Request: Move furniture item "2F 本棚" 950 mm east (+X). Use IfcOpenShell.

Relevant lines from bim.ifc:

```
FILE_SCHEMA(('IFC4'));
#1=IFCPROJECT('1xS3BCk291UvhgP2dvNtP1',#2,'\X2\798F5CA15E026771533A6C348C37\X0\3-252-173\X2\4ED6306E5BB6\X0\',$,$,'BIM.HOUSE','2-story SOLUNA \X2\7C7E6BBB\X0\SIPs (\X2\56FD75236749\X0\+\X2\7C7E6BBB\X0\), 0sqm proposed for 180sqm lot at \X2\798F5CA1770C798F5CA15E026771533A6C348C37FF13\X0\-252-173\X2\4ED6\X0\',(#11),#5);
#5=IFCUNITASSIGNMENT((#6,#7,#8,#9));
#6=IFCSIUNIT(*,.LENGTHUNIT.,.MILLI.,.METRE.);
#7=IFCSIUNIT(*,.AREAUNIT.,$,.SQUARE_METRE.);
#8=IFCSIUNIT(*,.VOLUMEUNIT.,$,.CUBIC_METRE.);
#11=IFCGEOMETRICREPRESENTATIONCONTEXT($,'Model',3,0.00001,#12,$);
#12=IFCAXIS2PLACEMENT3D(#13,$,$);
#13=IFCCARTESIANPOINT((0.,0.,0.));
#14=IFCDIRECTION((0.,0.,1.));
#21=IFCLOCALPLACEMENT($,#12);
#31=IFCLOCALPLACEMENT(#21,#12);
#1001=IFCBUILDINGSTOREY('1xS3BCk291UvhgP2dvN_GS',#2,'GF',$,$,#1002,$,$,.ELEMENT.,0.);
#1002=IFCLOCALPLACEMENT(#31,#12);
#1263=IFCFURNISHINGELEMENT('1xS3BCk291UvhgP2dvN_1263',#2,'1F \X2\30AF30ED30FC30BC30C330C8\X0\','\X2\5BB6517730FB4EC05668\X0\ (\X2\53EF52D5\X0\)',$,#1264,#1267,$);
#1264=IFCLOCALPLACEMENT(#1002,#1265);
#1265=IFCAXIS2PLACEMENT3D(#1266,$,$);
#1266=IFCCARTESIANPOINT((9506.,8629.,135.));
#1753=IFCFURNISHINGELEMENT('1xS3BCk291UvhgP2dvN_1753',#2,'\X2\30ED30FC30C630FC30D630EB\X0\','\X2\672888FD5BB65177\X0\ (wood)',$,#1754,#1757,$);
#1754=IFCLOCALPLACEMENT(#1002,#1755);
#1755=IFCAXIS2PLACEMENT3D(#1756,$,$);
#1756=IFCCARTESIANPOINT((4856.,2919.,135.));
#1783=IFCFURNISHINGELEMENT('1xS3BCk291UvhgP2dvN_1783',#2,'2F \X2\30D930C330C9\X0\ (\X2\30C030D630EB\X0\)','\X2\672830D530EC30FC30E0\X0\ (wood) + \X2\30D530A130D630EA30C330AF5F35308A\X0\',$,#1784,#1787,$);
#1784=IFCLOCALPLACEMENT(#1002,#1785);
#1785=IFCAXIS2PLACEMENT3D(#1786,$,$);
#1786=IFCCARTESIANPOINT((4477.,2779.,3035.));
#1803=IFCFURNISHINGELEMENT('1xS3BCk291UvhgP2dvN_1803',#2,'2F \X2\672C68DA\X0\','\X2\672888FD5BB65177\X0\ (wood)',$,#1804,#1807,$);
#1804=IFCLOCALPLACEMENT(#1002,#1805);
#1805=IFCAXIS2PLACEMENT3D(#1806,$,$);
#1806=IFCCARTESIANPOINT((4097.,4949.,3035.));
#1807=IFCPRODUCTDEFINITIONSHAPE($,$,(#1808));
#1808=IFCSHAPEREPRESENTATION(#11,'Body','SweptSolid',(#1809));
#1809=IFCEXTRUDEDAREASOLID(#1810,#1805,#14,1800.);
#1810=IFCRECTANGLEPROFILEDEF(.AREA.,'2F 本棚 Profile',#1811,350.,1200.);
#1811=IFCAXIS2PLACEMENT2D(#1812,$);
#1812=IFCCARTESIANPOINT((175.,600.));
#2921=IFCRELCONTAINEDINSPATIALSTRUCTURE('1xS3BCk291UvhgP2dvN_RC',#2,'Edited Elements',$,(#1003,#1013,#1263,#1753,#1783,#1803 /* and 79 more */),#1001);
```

```python
import ifcopenshell
import ifcopenshell.api.geometry
import ifcopenshell.util.placement
import ifcopenshell.util.unit

model = ifcopenshell.open("bim.ifc")
unit_scale = ifcopenshell.util.unit.calculate_unit_scale(model)

item = model.by_id(1803)
matrix = ifcopenshell.util.placement.get_local_placement(item.ObjectPlacement)
matrix[0, 3] += 0.95 / unit_scale
ifcopenshell.api.geometry.edit_object_placement(model, product=item, matrix=matrix, is_si=False)

print(ifcopenshell.util.placement.get_local_placement(item.ObjectPlacement).round(3) + 0.0)

model.write("bim-out.ifc")
```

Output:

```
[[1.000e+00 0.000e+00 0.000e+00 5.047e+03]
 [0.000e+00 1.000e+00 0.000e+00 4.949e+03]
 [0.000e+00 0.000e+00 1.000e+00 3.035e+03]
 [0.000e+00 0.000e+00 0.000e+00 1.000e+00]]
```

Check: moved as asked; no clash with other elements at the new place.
